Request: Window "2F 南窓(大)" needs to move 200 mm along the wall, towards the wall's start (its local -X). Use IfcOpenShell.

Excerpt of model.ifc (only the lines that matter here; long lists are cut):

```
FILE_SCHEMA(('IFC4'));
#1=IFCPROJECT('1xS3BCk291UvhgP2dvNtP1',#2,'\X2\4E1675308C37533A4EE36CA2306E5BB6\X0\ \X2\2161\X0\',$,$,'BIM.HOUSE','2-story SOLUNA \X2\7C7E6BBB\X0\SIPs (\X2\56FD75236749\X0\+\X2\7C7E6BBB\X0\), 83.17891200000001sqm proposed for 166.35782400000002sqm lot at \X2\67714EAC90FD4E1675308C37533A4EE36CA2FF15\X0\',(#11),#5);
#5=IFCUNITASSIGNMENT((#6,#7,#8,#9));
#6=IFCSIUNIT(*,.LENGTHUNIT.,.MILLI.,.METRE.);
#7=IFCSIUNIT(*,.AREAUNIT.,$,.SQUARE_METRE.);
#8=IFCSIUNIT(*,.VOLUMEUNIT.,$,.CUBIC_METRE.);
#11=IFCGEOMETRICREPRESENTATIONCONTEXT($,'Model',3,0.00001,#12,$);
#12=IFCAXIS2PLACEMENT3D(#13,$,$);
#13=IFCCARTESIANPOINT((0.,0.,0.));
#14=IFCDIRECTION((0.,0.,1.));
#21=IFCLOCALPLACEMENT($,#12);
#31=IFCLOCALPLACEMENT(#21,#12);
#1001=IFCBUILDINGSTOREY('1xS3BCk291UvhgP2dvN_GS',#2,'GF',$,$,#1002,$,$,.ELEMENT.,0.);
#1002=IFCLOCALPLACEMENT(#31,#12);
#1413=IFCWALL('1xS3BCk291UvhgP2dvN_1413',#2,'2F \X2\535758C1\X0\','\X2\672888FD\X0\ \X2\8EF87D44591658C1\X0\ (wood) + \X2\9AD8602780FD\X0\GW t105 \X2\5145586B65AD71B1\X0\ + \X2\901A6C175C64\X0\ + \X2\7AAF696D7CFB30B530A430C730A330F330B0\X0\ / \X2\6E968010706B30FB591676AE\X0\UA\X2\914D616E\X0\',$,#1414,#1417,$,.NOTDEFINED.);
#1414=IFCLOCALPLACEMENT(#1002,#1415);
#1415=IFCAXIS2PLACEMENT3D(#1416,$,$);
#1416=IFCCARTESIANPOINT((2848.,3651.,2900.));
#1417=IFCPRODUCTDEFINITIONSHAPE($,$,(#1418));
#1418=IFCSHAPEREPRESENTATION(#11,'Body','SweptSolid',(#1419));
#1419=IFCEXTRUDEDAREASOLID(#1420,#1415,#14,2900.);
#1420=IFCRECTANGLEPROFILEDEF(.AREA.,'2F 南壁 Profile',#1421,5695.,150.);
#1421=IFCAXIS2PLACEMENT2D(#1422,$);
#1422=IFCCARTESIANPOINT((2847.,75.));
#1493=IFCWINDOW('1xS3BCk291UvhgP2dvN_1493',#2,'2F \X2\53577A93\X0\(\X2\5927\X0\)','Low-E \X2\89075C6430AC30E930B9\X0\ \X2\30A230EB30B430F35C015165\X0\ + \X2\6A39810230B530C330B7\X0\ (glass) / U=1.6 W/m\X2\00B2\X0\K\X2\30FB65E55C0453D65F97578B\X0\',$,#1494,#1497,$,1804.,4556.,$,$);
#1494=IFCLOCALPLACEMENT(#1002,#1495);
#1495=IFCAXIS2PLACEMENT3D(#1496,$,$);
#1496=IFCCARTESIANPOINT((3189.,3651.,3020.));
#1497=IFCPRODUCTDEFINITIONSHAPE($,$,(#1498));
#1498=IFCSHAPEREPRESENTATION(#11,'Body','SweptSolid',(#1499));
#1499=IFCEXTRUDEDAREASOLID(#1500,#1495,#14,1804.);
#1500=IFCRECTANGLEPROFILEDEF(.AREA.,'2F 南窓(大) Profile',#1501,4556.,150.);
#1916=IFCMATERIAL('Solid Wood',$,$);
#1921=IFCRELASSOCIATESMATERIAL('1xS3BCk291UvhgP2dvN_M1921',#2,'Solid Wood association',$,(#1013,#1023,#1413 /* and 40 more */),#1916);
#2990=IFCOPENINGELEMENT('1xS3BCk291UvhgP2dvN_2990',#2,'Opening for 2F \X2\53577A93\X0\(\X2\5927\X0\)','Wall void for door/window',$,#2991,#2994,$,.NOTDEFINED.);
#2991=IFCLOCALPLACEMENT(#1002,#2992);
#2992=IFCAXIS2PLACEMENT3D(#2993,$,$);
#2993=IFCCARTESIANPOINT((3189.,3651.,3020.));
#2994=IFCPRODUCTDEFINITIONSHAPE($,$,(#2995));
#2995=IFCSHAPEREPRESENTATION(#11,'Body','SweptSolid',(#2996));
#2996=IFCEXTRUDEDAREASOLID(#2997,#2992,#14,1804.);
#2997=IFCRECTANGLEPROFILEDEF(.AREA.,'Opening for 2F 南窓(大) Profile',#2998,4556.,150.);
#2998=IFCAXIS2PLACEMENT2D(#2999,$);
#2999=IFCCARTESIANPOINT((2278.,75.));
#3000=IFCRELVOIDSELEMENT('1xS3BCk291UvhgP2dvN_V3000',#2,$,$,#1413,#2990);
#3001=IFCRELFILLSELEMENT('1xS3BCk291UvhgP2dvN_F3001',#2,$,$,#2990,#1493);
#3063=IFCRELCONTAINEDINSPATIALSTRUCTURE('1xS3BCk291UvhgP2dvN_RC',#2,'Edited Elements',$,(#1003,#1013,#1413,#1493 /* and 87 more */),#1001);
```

```python
import ifcopenshell
import ifcopenshell.api.geometry
import ifcopenshell.util.placement

model = ifcopenshell.open("model.ifc")

window = model.by_guid("1xS3BCk291UvhgP2dvN_1493")
opening = window.FillsVoids[0].RelatingOpeningElement
wall = opening.VoidsElements[0].RelatingBuildingElement

wall_matrix = ifcopenshell.util.placement.get_local_placement(wall.ObjectPlacement)
shift = wall_matrix[:3, 0] * -200.0
before = ifcopenshell.util.placement.get_local_placement(window.ObjectPlacement)[:3, 3].copy()

# The window is not placed relative to its opening, so move both.
for product in (opening, window):
    matrix = ifcopenshell.util.placement.get_local_placement(product.ObjectPlacement)
    matrix[:3, 3] += shift
    ifcopenshell.api.geometry.edit_object_placement(model, product=product, matrix=matrix, is_si=False)

after = ifcopenshell.util.placement.get_local_placement(window.ObjectPlacement)[:3, 3]
print("window moved by", (after - before).round(3) + 0.0)

model.write("model-out.ifc")
```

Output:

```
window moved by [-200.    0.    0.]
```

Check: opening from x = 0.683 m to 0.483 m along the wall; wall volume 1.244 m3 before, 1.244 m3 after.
